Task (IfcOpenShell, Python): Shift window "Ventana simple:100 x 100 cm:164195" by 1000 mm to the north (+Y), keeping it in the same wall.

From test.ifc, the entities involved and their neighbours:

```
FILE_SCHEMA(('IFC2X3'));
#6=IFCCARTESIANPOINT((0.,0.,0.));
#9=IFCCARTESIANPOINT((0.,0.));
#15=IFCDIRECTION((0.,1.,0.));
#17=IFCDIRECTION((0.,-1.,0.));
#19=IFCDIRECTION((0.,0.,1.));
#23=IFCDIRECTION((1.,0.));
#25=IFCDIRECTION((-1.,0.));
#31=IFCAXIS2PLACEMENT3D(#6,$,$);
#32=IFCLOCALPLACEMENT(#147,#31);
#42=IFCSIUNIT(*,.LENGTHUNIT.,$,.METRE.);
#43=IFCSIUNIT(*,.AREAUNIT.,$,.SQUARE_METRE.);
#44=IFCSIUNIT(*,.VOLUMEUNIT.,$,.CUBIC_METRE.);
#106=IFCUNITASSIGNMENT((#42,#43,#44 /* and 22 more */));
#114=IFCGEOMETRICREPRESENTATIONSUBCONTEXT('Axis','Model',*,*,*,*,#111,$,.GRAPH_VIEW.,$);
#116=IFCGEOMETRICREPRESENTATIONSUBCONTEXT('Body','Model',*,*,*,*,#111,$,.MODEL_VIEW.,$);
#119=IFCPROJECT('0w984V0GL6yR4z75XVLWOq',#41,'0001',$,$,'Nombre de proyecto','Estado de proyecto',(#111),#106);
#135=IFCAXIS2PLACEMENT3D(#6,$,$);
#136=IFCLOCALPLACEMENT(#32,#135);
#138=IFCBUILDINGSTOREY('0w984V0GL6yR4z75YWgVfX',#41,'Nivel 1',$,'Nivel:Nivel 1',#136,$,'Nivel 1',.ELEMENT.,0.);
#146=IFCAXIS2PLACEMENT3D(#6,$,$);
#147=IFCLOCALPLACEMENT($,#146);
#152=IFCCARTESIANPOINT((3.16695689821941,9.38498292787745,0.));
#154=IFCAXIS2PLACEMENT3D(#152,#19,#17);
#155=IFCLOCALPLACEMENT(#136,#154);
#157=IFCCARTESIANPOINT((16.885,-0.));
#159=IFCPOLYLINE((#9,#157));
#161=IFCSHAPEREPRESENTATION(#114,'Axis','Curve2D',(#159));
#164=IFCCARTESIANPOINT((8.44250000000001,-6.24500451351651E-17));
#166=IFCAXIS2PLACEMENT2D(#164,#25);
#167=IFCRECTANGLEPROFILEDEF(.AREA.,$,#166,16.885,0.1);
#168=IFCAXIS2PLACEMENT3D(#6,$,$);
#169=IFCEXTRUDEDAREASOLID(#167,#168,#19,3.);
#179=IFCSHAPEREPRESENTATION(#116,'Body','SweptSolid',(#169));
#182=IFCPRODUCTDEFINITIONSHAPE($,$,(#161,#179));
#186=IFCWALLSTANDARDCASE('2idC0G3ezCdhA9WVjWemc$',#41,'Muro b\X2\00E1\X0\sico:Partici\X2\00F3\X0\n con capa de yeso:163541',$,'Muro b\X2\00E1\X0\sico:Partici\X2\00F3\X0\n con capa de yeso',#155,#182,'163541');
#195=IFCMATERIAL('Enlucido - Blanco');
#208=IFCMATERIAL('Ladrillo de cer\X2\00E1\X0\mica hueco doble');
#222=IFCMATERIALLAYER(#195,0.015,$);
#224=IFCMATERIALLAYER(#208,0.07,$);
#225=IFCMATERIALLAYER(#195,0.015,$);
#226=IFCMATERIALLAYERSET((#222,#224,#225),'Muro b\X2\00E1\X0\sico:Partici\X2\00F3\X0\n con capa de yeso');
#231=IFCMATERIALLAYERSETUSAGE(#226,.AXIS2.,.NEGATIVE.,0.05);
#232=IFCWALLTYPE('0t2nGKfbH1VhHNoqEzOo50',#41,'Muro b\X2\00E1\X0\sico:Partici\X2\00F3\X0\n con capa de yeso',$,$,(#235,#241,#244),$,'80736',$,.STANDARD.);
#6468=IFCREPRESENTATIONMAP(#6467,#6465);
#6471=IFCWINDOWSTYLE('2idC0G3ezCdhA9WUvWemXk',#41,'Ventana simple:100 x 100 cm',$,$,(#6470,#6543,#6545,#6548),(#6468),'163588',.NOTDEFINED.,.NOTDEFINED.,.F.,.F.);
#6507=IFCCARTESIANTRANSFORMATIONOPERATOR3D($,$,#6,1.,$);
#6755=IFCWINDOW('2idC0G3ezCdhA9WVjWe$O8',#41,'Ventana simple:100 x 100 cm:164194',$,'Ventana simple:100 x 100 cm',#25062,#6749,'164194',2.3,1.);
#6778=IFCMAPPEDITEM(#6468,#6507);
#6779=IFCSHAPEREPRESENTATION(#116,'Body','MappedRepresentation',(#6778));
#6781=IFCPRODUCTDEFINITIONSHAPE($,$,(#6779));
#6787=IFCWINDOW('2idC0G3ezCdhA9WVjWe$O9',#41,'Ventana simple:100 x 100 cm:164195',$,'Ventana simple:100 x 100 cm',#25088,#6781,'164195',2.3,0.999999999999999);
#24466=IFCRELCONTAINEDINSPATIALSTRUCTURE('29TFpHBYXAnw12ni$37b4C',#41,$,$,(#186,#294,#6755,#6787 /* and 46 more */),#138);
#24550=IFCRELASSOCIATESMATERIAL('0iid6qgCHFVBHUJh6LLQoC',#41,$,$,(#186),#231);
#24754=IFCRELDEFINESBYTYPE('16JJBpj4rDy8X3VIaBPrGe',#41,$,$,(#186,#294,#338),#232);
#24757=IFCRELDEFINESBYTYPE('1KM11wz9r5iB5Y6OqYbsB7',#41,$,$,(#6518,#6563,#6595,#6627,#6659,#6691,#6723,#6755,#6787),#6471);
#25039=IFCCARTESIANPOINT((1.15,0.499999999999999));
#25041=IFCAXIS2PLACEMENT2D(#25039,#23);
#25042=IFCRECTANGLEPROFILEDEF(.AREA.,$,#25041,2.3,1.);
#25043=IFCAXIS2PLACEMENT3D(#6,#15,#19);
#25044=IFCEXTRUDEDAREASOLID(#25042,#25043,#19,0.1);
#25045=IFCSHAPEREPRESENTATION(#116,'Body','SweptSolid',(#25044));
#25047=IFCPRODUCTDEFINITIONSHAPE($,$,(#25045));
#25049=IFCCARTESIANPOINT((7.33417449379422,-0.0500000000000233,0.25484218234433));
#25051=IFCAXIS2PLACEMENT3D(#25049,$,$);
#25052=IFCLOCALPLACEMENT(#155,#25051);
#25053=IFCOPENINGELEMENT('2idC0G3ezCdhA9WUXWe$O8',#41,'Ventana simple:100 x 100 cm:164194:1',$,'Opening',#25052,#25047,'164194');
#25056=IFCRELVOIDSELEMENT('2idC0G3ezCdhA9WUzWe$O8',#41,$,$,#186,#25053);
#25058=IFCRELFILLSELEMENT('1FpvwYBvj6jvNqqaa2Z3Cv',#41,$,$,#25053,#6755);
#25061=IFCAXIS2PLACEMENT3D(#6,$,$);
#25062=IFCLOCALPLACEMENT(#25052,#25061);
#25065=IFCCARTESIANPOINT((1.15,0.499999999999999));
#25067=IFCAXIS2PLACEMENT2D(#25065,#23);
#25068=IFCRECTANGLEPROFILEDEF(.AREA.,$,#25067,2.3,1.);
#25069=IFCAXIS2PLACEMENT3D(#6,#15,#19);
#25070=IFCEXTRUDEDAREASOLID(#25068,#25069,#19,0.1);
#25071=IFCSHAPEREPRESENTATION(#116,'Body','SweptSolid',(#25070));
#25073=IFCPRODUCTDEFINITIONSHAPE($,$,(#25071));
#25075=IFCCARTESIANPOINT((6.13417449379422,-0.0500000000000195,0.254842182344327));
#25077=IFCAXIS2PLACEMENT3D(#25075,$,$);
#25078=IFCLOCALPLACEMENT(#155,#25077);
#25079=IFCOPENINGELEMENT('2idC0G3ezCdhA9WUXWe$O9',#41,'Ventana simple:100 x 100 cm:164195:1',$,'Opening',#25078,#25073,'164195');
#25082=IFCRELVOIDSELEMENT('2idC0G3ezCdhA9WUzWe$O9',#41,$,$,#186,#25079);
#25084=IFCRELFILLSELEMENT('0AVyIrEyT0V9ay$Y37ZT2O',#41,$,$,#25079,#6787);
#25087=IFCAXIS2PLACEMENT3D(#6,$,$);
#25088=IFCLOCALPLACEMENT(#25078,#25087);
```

```python
import ifcopenshell
import ifcopenshell.api.geometry
import ifcopenshell.util.placement
import ifcopenshell.util.unit

model = ifcopenshell.open("test.ifc")
unit_scale = ifcopenshell.util.unit.calculate_unit_scale(model)

window = model.by_id(6787)
opening = window.FillsVoids[0].RelatingOpeningElement
wall = opening.VoidsElements[0].RelatingBuildingElement

wall_matrix = ifcopenshell.util.placement.get_local_placement(wall.ObjectPlacement)
shift = wall_matrix[:3, 0] * -1 / unit_scale
before = ifcopenshell.util.placement.get_local_placement(window.ObjectPlacement)[:3, 3].copy()

# The window is placed relative to its opening, so it follows when the opening moves.
matrix = ifcopenshell.util.placement.get_local_placement(opening.ObjectPlacement)
matrix[:3, 3] += shift
ifcopenshell.api.geometry.edit_object_placement(
    model, product=opening, matrix=matrix, is_si=False, should_transform_children=True
)

after = ifcopenshell.util.placement.get_local_placement(window.ObjectPlacement)[:3, 3]
print("window moved by", (after - before).round(3) + 0.0)

model.write("test_updated.ifc")
```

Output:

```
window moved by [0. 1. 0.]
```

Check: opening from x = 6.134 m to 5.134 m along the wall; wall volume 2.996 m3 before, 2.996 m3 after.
